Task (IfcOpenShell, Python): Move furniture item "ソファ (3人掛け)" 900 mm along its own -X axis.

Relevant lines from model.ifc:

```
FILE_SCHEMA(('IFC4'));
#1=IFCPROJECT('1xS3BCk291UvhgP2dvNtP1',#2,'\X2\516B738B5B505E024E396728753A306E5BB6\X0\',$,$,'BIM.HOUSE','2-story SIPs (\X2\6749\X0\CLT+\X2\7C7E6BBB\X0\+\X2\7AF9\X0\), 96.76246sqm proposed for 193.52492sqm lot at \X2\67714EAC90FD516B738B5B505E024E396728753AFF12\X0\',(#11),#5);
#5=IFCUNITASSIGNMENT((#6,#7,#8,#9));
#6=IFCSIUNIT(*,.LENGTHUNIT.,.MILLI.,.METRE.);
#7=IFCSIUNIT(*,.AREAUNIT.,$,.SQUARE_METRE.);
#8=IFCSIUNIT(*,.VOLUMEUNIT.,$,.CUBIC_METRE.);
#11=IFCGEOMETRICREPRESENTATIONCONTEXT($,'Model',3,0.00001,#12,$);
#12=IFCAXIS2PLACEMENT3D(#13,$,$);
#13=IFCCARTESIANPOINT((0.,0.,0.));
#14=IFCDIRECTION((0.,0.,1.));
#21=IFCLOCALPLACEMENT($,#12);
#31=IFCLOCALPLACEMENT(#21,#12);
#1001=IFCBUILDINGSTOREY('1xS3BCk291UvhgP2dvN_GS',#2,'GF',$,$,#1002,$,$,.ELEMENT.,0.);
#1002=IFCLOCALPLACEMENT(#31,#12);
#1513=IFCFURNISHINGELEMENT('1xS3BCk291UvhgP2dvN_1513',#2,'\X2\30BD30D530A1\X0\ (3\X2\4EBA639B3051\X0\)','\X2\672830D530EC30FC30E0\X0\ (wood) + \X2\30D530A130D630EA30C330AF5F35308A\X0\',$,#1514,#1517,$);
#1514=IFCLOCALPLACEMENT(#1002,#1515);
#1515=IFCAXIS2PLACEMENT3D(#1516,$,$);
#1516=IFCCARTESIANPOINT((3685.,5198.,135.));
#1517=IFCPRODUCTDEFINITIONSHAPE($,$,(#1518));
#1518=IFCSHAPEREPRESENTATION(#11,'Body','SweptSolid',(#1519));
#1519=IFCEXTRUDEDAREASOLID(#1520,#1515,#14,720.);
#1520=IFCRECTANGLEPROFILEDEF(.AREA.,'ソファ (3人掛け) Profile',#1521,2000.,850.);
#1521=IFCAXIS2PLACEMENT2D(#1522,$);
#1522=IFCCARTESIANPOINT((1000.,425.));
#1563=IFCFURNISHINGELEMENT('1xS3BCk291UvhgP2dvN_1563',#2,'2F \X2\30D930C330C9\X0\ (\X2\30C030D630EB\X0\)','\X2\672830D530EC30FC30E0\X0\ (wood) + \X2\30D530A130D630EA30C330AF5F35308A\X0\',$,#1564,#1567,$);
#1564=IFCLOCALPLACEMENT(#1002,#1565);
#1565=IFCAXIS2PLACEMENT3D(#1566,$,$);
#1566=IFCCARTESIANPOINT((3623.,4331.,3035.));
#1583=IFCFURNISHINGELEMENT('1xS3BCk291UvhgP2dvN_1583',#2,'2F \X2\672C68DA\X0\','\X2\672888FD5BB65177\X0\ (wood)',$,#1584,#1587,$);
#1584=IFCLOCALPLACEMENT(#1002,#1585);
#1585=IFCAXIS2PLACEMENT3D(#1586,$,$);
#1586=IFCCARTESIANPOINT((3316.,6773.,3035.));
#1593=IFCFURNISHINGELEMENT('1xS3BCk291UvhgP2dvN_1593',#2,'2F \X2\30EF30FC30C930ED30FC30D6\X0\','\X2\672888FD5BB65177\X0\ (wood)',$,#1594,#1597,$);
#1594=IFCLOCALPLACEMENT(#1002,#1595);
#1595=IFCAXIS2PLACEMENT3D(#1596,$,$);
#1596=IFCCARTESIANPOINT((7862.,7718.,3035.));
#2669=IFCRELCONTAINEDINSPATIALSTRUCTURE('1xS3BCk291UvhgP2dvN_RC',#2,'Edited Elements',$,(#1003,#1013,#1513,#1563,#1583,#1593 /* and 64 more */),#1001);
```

```python
import ifcopenshell
import ifcopenshell.api.geometry
import ifcopenshell.util.placement
import ifcopenshell.util.unit

model = ifcopenshell.open("model.ifc")
unit_scale = ifcopenshell.util.unit.calculate_unit_scale(model)

item = model.by_id(1513)
matrix = ifcopenshell.util.placement.get_local_placement(item.ObjectPlacement)
matrix[:3, 3] -= matrix[:3, 0] * 0.9 / unit_scale
ifcopenshell.api.geometry.edit_object_placement(model, product=item, matrix=matrix, is_si=False)

print(ifcopenshell.util.placement.get_local_placement(item.ObjectPlacement).round(3) + 0.0)

model.write("model_updated.ifc")
```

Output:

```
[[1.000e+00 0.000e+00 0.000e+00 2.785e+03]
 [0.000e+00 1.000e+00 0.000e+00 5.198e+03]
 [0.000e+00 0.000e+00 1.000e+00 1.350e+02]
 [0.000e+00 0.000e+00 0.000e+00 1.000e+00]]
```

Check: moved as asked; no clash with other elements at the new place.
